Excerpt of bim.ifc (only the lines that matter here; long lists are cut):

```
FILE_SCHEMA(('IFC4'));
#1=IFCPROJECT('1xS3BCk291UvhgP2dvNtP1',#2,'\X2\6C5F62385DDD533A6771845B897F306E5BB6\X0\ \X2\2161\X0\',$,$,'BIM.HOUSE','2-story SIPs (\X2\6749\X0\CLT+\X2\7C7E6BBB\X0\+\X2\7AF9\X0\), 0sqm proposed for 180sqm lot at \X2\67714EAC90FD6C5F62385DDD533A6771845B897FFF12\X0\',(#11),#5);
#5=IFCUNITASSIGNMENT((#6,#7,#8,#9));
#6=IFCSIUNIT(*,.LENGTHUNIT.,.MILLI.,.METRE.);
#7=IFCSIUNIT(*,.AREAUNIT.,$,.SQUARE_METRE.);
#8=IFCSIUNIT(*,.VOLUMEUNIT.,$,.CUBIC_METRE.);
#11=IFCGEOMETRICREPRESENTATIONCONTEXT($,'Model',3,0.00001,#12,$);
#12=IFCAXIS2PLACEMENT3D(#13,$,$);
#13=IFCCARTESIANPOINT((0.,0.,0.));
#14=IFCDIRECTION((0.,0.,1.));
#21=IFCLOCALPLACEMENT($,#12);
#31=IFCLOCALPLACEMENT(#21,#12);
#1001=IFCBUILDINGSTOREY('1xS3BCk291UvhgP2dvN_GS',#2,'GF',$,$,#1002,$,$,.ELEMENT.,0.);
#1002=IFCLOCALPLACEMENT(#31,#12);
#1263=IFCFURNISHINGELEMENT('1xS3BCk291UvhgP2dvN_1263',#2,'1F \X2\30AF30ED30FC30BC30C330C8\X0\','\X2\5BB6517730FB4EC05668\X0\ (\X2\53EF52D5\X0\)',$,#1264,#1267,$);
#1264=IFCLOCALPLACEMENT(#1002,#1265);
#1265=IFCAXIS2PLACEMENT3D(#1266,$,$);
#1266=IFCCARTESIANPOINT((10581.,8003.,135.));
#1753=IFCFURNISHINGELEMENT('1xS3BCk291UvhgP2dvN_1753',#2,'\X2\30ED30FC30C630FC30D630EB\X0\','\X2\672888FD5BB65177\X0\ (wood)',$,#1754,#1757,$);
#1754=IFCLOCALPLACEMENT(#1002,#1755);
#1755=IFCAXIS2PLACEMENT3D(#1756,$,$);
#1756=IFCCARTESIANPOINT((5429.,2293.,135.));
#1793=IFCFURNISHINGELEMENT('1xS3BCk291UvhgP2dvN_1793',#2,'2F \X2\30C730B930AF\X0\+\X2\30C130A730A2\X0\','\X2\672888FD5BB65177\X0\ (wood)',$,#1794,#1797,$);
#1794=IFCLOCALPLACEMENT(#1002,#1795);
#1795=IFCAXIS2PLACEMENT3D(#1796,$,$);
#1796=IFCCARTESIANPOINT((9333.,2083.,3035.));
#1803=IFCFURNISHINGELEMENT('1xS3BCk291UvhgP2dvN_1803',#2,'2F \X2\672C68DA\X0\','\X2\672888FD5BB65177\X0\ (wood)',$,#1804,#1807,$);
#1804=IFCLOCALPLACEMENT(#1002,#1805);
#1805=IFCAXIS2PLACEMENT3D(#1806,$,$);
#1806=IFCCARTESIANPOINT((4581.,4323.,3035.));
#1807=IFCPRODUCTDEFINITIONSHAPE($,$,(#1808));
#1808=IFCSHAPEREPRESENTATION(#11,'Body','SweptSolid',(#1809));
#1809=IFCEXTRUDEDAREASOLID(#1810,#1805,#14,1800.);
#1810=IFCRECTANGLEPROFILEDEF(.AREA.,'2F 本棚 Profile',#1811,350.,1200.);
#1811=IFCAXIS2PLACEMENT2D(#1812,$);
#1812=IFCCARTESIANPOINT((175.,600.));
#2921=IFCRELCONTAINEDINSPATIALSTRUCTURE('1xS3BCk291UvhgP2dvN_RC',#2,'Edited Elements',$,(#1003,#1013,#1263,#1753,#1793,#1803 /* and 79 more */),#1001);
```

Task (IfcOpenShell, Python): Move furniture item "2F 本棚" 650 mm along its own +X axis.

```python
import ifcopenshell
import ifcopenshell.api.geometry
import ifcopenshell.util.placement
import ifcopenshell.util.unit

model = ifcopenshell.open("bim.ifc")
unit_scale = ifcopenshell.util.unit.calculate_unit_scale(model)

item = model.by_guid("1xS3BCk291UvhgP2dvN_1803")
matrix = ifcopenshell.util.placement.get_local_placement(item.ObjectPlacement)
matrix[:3, 3] += matrix[:3, 0] * 0.65 / unit_scale
ifcopenshell.api.geometry.edit_object_placement(model, product=item, matrix=matrix, is_si=False)

print(ifcopenshell.util.placement.get_local_placement(item.ObjectPlacement).round(3) + 0.0)

model.write("bim_v2.ifc")
```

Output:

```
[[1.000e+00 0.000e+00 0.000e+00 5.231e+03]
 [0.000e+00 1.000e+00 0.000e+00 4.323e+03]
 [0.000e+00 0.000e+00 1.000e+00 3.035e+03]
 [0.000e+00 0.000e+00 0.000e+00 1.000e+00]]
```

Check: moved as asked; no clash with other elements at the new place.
